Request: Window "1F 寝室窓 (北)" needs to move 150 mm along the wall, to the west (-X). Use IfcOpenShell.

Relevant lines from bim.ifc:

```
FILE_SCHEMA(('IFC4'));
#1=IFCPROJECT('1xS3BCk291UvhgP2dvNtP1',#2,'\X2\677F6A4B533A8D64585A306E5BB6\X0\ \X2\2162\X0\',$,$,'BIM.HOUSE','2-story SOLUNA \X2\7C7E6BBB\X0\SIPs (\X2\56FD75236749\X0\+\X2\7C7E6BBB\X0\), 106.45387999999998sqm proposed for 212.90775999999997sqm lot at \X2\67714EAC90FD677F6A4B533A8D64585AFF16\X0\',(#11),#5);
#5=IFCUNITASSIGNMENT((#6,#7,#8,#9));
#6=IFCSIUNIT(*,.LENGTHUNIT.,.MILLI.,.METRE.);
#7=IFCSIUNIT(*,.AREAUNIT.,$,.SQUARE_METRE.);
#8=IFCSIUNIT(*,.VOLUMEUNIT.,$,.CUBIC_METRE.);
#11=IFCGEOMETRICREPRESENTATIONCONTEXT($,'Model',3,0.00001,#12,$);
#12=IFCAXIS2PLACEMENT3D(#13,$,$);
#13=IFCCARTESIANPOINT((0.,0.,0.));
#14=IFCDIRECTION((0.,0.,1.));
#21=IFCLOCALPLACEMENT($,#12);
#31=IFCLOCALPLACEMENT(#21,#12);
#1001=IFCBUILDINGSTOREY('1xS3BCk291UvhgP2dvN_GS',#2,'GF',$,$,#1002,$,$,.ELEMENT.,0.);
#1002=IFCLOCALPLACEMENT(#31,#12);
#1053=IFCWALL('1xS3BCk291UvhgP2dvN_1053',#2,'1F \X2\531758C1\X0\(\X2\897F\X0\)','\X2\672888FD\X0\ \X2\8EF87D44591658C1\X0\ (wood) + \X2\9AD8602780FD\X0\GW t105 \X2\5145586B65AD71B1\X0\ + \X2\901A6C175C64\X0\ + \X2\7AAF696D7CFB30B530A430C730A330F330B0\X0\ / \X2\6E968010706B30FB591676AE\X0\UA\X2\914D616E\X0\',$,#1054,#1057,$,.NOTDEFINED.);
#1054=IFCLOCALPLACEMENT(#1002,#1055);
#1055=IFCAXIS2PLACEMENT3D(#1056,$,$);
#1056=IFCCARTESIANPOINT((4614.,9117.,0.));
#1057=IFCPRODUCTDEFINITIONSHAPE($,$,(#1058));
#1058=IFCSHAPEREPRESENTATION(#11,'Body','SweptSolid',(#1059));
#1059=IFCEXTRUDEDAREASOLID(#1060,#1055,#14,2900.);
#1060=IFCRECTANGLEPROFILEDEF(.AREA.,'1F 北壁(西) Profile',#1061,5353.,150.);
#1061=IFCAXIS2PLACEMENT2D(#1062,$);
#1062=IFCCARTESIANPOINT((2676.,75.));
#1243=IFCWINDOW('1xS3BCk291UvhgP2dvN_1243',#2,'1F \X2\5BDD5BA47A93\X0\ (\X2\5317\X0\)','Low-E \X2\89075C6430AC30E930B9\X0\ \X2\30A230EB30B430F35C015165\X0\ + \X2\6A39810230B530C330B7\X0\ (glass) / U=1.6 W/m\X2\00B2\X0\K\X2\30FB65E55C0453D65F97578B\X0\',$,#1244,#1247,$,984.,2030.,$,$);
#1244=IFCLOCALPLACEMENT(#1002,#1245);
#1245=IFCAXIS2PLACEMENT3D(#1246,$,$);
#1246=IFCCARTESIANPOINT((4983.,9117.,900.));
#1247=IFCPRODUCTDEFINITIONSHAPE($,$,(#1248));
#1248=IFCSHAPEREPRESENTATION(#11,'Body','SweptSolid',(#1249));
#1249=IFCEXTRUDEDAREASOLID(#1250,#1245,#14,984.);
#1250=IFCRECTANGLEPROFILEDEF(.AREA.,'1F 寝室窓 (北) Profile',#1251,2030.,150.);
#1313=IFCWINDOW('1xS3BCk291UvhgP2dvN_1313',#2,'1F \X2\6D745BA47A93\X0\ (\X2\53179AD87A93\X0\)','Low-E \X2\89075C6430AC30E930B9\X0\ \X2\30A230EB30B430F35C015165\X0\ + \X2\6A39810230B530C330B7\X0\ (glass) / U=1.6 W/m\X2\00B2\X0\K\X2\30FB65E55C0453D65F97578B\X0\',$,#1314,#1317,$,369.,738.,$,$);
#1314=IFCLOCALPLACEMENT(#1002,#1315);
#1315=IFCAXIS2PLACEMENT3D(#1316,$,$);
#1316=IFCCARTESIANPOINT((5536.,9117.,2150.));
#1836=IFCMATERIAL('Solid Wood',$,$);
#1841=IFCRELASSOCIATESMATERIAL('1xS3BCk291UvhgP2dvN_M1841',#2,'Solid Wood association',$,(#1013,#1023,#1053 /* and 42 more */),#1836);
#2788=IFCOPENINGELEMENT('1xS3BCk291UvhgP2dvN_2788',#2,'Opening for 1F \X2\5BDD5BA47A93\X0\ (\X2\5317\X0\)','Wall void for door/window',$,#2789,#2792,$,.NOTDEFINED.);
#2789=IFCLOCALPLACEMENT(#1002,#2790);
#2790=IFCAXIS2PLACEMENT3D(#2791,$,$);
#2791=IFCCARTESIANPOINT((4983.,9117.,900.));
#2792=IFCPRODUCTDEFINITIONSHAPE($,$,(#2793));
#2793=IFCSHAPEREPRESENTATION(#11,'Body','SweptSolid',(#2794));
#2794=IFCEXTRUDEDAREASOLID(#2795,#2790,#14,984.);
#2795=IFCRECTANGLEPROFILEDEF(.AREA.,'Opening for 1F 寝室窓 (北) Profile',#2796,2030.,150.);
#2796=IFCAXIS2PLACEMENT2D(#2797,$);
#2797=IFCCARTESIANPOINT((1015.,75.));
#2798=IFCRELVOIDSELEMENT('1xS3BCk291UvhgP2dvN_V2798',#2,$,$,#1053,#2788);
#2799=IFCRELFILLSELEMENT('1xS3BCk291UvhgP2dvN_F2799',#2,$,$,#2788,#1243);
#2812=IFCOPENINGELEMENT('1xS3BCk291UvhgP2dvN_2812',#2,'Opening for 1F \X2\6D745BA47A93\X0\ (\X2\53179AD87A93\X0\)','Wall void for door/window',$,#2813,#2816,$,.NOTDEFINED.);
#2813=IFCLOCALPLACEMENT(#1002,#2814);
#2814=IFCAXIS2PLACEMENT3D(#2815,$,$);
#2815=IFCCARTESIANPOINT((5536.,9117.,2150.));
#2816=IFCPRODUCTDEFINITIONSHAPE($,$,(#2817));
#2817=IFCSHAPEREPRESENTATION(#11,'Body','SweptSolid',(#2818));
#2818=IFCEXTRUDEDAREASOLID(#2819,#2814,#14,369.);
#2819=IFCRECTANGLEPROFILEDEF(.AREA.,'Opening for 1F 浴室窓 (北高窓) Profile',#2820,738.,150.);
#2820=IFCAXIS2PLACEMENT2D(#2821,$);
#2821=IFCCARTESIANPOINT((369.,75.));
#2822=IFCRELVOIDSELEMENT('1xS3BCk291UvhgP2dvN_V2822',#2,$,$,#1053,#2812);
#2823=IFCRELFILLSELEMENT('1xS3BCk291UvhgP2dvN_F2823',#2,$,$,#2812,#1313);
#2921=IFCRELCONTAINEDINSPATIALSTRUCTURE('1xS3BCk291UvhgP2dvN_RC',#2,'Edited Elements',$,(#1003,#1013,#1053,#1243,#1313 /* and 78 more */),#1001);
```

```python
import ifcopenshell
import ifcopenshell.api.geometry
import ifcopenshell.util.placement
import ifcopenshell.util.unit

model = ifcopenshell.open("bim.ifc")
unit_scale = ifcopenshell.util.unit.calculate_unit_scale(model)

window = model.by_guid("1xS3BCk291UvhgP2dvN_1243")
opening = window.FillsVoids[0].RelatingOpeningElement
wall = opening.VoidsElements[0].RelatingBuildingElement

wall_matrix = ifcopenshell.util.placement.get_local_placement(wall.ObjectPlacement)
shift = wall_matrix[:3, 0] * -0.15 / unit_scale
before = ifcopenshell.util.placement.get_local_placement(window.ObjectPlacement)[:3, 3].copy()

# The window is not placed relative to its opening, so move both.
for product in (opening, window):
    matrix = ifcopenshell.util.placement.get_local_placement(product.ObjectPlacement)
    matrix[:3, 3] += shift
    ifcopenshell.api.geometry.edit_object_placement(model, product=product, matrix=matrix, is_si=False)

after = ifcopenshell.util.placement.get_local_placement(window.ObjectPlacement)[:3, 3]
print("window moved by", (after - before).round(3) + 0.0)

model.write("bim-out.ifc")
```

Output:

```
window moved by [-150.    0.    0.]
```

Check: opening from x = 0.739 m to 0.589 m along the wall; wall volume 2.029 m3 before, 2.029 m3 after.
